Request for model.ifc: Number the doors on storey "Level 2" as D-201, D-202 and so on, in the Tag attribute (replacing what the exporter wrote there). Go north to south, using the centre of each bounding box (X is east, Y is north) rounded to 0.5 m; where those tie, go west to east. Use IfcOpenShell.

First a look at what the model holds.

```python
import ifcopenshell
import ifcopenshell.util.element
import ifcopenshell.util.placement

model = ifcopenshell.open("model.ifc")
print(model.schema)
storey = next(s for s in model.by_type("IfcBuildingStorey") if s.Name == "Level 2")
doors = [e for e in ifcopenshell.util.element.get_decomposition(storey) if e.is_a("IfcDoor")]
for e in sorted(doors, key=lambda e: e.id()):
    origin = ifcopenshell.util.placement.get_local_placement(e.ObjectPlacement)[:3, 3]
    print(e.id(), e.Tag, e.Name, origin.round(2) + 0.0, sep=" | ")
```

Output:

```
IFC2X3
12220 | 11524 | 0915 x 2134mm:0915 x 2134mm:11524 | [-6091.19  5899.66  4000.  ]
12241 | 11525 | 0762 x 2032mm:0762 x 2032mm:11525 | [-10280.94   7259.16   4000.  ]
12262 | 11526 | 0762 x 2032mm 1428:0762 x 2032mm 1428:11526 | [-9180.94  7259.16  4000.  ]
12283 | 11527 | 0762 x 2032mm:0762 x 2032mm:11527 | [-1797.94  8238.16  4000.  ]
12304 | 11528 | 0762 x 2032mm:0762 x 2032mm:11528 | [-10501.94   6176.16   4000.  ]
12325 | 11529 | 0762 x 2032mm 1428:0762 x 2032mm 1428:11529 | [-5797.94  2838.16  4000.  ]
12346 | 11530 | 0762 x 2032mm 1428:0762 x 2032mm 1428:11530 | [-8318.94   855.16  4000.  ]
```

```python
import ifcopenshell
import ifcopenshell.geom
import ifcopenshell.util.element
import ifcopenshell.util.shape

model = ifcopenshell.open("model.ifc")
settings = ifcopenshell.geom.settings()
settings.set("use-world-coords", True)


def centre(element):
    shape = ifcopenshell.geom.create_shape(settings, element)
    return ifcopenshell.util.shape.get_bbox_centroid(shape.geometry)


storey = next(s for s in model.by_type("IfcBuildingStorey") if s.Name == "Level 2")
doors = [e for e in ifcopenshell.util.element.get_decomposition(storey) if e.is_a("IfcDoor")]

# Insertion points can sit at a corner or the storey origin, so sort by the geometry (in metres).
centres = {e: centre(e) for e in doors}
doors.sort(key=lambda e: (-round(centres[e][1] / 0.5), centres[e][0]))

for i, e in enumerate(doors, start=1):
    number = f"D-2{i:02d}"
    e.Tag = number
    print(e.id(), number)

model.write("model_v2.ifc")
```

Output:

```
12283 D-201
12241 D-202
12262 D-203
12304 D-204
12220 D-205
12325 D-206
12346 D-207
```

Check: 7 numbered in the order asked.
